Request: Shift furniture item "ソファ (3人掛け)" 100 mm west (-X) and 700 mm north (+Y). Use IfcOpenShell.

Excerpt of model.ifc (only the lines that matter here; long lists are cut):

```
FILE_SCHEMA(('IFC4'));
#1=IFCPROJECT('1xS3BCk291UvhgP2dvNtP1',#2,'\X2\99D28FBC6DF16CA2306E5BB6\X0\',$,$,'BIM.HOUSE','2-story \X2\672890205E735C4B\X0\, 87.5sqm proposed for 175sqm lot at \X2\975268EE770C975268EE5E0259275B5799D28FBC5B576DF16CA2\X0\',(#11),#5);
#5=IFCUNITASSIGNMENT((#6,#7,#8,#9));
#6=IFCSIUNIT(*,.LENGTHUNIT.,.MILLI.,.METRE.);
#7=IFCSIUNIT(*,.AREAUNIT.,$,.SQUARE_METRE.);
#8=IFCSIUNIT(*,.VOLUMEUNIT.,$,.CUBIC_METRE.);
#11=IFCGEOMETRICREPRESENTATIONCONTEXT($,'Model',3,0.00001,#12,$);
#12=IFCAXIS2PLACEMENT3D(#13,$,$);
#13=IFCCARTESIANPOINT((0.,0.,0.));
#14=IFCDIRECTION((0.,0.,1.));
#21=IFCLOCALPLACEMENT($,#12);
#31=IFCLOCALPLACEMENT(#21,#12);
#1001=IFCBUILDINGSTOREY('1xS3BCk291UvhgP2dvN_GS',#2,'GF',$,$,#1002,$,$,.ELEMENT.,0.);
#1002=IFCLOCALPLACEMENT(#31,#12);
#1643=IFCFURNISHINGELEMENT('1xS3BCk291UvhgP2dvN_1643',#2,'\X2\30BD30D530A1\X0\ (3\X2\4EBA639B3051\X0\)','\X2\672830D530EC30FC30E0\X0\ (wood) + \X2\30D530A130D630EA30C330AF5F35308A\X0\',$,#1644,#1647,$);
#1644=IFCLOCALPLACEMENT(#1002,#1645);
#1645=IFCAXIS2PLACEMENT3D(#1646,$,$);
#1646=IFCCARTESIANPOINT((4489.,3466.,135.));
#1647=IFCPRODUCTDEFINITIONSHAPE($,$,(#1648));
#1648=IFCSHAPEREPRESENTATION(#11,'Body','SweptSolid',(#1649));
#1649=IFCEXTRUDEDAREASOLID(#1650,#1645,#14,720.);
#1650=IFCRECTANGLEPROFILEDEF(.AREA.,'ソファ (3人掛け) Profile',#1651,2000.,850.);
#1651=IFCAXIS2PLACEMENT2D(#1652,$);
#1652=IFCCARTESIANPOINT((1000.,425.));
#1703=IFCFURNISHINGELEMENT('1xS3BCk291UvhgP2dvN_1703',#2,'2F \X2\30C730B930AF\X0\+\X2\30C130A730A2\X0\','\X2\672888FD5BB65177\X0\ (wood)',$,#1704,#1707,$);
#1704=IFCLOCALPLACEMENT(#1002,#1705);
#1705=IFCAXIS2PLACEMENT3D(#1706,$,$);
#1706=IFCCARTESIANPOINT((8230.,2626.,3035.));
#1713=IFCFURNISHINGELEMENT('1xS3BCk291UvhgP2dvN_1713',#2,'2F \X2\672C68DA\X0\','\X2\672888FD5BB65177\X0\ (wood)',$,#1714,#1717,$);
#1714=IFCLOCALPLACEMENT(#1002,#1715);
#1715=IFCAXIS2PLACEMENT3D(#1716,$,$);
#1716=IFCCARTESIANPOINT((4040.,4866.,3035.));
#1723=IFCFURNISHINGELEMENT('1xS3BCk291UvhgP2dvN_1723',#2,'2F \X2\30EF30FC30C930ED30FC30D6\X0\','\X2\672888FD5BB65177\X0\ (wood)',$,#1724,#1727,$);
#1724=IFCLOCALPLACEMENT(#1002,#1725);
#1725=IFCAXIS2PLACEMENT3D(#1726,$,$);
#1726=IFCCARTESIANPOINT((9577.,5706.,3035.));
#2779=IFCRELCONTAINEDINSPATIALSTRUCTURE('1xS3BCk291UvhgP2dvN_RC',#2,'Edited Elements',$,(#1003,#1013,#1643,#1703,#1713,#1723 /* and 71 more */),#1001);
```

```python
import ifcopenshell
import ifcopenshell.api.geometry
import ifcopenshell.util.placement
import ifcopenshell.util.unit

model = ifcopenshell.open("model.ifc")
unit_scale = ifcopenshell.util.unit.calculate_unit_scale(model)

item = model.by_guid("1xS3BCk291UvhgP2dvN_1643")
matrix = ifcopenshell.util.placement.get_local_placement(item.ObjectPlacement)
matrix[0, 3] -= 0.1 / unit_scale
matrix[1, 3] += 0.7 / unit_scale
ifcopenshell.api.geometry.edit_object_placement(model, product=item, matrix=matrix, is_si=False)

print(ifcopenshell.util.placement.get_local_placement(item.ObjectPlacement).round(3) + 0.0)

model.write("model_rev.ifc")
```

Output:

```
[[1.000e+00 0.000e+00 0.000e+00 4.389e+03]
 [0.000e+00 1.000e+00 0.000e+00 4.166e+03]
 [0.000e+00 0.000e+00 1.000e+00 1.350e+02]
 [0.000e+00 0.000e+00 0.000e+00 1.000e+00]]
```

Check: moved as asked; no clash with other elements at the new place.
